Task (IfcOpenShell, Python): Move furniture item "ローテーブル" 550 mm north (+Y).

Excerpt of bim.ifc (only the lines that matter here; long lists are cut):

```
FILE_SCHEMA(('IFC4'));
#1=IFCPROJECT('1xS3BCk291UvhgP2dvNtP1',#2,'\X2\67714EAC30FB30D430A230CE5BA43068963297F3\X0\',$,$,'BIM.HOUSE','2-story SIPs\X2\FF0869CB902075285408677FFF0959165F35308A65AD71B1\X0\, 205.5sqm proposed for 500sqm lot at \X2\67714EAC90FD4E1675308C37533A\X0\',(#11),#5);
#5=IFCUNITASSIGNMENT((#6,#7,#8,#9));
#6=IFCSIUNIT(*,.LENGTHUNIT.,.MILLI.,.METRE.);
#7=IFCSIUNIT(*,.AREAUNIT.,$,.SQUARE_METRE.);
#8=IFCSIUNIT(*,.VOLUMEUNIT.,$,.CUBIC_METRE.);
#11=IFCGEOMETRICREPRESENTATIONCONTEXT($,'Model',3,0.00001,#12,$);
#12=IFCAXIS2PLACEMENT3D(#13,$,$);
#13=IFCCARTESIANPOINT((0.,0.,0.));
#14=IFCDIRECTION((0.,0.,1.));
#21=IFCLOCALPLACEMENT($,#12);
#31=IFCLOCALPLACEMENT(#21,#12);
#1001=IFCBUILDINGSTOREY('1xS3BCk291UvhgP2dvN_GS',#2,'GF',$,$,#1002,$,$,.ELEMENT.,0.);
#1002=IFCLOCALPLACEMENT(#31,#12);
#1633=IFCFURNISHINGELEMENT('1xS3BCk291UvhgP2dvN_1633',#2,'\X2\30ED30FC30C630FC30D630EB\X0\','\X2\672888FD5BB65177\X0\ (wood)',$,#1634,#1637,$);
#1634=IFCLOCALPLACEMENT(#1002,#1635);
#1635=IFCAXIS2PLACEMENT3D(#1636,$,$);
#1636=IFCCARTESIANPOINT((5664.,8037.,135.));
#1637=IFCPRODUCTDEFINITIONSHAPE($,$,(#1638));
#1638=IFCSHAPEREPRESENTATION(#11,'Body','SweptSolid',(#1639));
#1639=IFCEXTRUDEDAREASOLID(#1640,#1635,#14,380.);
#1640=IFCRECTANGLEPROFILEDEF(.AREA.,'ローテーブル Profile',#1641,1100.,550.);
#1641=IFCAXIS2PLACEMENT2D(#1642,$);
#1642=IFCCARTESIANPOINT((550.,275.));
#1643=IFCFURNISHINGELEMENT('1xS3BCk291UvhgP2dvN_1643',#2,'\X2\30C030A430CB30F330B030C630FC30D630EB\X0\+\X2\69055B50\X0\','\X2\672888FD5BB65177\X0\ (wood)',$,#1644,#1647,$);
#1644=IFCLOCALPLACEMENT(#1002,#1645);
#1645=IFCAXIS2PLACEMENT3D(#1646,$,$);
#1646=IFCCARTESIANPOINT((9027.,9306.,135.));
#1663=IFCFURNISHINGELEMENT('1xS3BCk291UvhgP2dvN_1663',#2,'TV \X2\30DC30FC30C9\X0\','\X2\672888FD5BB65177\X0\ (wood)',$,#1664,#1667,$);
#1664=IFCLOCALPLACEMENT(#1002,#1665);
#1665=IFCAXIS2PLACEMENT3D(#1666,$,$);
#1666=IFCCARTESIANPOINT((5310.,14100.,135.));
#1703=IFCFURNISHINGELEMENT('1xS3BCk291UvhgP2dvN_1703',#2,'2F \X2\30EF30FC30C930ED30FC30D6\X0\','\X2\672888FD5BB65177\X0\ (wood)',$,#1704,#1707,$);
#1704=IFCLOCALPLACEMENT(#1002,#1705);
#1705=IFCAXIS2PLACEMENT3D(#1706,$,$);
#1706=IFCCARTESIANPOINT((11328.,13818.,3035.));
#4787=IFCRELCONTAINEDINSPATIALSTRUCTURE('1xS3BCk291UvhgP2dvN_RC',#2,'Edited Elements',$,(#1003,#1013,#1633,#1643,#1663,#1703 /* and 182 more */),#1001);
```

```python
import ifcopenshell
import ifcopenshell.api.geometry
import ifcopenshell.util.placement
import ifcopenshell.util.unit

model = ifcopenshell.open("bim.ifc")
unit_scale = ifcopenshell.util.unit.calculate_unit_scale(model)

item = model.by_guid("1xS3BCk291UvhgP2dvN_1633")
matrix = ifcopenshell.util.placement.get_local_placement(item.ObjectPlacement)
matrix[1, 3] += 0.55 / unit_scale
ifcopenshell.api.geometry.edit_object_placement(model, product=item, matrix=matrix, is_si=False)

print(ifcopenshell.util.placement.get_local_placement(item.ObjectPlacement).round(3) + 0.0)

model.write("bim_edited.ifc")
```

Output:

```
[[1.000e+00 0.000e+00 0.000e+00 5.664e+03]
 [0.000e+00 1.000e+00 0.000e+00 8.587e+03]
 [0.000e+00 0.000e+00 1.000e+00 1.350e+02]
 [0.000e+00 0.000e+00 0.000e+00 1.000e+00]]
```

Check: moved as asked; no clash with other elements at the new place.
